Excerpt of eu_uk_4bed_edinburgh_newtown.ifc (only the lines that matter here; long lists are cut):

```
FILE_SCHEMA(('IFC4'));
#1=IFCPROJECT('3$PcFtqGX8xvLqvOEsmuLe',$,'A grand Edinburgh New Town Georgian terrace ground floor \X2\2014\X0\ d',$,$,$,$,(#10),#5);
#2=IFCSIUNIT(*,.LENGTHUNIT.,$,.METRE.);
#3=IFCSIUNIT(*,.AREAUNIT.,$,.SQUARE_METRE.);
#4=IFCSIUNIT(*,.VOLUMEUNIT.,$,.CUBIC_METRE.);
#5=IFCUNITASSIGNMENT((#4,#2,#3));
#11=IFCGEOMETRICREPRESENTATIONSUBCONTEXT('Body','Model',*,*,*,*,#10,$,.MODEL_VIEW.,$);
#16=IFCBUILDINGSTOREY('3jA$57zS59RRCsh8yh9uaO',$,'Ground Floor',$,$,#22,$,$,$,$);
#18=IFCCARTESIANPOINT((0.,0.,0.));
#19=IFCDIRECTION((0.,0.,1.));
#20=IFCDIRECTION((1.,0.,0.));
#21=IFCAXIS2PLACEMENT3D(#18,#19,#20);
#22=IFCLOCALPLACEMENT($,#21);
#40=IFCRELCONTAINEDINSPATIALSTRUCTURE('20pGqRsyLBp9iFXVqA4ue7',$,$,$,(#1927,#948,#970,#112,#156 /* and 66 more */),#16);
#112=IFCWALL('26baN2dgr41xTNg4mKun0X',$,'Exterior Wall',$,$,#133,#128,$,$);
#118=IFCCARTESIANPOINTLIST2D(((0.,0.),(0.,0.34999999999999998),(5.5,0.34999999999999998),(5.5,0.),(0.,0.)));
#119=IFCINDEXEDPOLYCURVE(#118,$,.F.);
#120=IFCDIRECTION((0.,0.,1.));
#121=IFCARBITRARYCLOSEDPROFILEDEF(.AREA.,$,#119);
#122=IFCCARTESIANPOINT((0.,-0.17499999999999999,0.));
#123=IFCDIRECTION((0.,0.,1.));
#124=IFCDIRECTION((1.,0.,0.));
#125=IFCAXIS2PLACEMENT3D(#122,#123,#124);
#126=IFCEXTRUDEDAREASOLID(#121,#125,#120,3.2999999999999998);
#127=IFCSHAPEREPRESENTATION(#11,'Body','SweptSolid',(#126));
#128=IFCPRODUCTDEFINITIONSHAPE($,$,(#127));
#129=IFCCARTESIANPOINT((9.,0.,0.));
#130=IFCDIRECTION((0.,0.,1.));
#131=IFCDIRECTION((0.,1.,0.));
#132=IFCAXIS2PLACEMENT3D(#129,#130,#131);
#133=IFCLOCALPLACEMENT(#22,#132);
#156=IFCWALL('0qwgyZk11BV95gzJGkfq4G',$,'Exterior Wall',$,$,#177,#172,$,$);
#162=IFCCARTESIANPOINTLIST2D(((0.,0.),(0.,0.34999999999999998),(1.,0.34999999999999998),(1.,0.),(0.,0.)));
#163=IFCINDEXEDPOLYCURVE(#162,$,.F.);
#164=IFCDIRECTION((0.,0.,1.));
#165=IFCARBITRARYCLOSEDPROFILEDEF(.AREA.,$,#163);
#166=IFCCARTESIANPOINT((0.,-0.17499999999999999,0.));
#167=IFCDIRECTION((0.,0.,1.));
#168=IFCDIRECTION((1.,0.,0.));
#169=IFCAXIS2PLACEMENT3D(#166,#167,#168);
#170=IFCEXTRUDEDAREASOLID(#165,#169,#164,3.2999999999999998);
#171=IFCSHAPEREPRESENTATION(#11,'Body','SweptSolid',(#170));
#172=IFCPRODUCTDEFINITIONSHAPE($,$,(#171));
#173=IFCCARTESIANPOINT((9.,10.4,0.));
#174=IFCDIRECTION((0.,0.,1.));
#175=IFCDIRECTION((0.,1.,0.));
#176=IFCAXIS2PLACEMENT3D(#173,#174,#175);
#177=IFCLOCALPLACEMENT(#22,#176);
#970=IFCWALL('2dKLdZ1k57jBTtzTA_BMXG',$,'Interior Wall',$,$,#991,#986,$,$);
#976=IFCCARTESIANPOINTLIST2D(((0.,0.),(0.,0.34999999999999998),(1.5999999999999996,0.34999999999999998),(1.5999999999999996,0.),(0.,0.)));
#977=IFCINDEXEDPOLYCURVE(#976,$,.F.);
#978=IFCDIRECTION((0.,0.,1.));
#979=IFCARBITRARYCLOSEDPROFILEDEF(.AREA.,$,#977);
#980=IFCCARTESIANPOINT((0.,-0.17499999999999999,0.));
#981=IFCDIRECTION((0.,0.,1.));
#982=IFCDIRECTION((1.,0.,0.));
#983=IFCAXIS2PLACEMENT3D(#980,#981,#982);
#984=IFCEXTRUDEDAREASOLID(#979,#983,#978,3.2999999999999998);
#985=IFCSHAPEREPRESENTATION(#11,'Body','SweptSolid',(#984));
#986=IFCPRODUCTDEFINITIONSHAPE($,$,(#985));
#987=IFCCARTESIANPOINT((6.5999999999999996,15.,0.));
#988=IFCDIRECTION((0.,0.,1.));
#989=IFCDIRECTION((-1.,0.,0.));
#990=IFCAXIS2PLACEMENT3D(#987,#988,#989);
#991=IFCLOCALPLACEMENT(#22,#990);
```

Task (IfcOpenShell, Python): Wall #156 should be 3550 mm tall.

```python
import ifcopenshell
import ifcopenshell.geom
import ifcopenshell.util.representation
import ifcopenshell.util.shape
import ifcopenshell.util.unit

model = ifcopenshell.open("eu_uk_4bed_edinburgh_newtown.ifc")
unit_scale = ifcopenshell.util.unit.calculate_unit_scale(model)
settings = ifcopenshell.geom.settings()


def volume(element):
    """Net volume in cubic metres, openings subtracted."""
    shape = ifcopenshell.geom.create_shape(settings, element)
    return ifcopenshell.util.shape.get_volume(shape.geometry)


wall = model.by_guid("0qwgyZk11BV95gzJGkfq4G")
before = volume(wall)

body = ifcopenshell.util.representation.get_representation(wall, "Model", "Body")
solid = body.Items[0]
old_height = solid.Depth
solid.Depth = 3.55 / unit_scale
after = volume(wall)

print(f"height {old_height:g} -> {solid.Depth:g}, volume {before:.3f} -> {after:.3f} m3")

model.write("eu_uk_4bed_edinburgh_newtown_edited.ifc")
```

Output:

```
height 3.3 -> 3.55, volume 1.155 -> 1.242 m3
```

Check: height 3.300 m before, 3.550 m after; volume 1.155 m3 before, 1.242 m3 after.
